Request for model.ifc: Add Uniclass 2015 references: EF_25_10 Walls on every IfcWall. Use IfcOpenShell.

First a look at what the model holds.

```python
import ifcopenshell

model = ifcopenshell.open("model.ifc")
print(model.schema)
print("classifications:", [c.Name for c in model.by_type("IfcClassification")])
for ifc_class in ("IfcDoor", "IfcRoof", "IfcStair", "IfcWall", "IfcWindow"):
    print(ifc_class, len(model.by_type(ifc_class)))
```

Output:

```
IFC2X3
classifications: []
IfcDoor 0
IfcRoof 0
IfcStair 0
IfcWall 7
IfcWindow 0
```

```python
import ifcopenshell
import ifcopenshell.api.classification

model = ifcopenshell.open("model.ifc")

# IFC2X3 requires Source and Edition and has no link from the project to the system.
system = model.create_entity("IfcClassification", Source="NBS", Edition="2015", Name="Uniclass 2015")

codes = {
    "IfcWall": ("EF_25_10", "Walls"),
}
for ifc_class, (code, name) in codes.items():
    products = model.by_type(ifc_class)
    ifcopenshell.api.classification.add_reference(
        model, products=products, classification=system, identification=code, name=name
    )
    print(code, len(products))

model.write("model_v2.ifc")
```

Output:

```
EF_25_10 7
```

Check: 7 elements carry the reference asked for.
